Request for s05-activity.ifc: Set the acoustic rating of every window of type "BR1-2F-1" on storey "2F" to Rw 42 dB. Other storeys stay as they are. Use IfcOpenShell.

First a look at what the model holds.

```python
import ifcopenshell
import ifcopenshell.util.element

model = ifcopenshell.open("s05-activity.ifc")
print(model.schema)
storey = next(s for s in model.by_type("IfcBuildingStorey") if s.Name == "2F")
windows = [e for e in ifcopenshell.util.element.get_decomposition(storey) if e.is_a("IfcWindow")]
seen = {}
for e in windows:
    element_type = ifcopenshell.util.element.get_type(e)
    key = (element_type.Name if element_type != e and element_type else None, ifcopenshell.util.element.get_pset(e, "Pset_WindowCommon", "AcousticRating"))
    seen[key] = seen.get(key, 0) + 1
for (name, value), count in sorted(seen.items(), key=str):
    print(count, "x", name, "|", value)
```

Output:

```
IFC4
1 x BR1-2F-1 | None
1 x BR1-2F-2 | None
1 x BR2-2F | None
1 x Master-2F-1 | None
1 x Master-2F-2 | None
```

```python
import ifcopenshell
import ifcopenshell.api.pset
import ifcopenshell.util.element

model = ifcopenshell.open("s05-activity.ifc")

storey = next(s for s in model.by_type("IfcBuildingStorey") if s.Name == "2F")
windows = [e for e in ifcopenshell.util.element.get_decomposition(storey) if e.is_a("IfcWindow")]

count = 0
for e in windows:
    element_type = ifcopenshell.util.element.get_type(e)
    if element_type in (None, e) or element_type.Name != "BR1-2F-1":
        continue
    # add_pset returns the element's existing set when there is one.
    pset = ifcopenshell.api.pset.add_pset(model, product=e, name="Pset_WindowCommon")
    ifcopenshell.api.pset.edit_pset(model, pset=pset, properties={"AcousticRating": "Rw 42 dB"})
    count += 1

print(count, "windows updated")

model.write("s05-activity_updated.ifc")
```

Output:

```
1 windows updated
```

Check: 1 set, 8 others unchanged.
